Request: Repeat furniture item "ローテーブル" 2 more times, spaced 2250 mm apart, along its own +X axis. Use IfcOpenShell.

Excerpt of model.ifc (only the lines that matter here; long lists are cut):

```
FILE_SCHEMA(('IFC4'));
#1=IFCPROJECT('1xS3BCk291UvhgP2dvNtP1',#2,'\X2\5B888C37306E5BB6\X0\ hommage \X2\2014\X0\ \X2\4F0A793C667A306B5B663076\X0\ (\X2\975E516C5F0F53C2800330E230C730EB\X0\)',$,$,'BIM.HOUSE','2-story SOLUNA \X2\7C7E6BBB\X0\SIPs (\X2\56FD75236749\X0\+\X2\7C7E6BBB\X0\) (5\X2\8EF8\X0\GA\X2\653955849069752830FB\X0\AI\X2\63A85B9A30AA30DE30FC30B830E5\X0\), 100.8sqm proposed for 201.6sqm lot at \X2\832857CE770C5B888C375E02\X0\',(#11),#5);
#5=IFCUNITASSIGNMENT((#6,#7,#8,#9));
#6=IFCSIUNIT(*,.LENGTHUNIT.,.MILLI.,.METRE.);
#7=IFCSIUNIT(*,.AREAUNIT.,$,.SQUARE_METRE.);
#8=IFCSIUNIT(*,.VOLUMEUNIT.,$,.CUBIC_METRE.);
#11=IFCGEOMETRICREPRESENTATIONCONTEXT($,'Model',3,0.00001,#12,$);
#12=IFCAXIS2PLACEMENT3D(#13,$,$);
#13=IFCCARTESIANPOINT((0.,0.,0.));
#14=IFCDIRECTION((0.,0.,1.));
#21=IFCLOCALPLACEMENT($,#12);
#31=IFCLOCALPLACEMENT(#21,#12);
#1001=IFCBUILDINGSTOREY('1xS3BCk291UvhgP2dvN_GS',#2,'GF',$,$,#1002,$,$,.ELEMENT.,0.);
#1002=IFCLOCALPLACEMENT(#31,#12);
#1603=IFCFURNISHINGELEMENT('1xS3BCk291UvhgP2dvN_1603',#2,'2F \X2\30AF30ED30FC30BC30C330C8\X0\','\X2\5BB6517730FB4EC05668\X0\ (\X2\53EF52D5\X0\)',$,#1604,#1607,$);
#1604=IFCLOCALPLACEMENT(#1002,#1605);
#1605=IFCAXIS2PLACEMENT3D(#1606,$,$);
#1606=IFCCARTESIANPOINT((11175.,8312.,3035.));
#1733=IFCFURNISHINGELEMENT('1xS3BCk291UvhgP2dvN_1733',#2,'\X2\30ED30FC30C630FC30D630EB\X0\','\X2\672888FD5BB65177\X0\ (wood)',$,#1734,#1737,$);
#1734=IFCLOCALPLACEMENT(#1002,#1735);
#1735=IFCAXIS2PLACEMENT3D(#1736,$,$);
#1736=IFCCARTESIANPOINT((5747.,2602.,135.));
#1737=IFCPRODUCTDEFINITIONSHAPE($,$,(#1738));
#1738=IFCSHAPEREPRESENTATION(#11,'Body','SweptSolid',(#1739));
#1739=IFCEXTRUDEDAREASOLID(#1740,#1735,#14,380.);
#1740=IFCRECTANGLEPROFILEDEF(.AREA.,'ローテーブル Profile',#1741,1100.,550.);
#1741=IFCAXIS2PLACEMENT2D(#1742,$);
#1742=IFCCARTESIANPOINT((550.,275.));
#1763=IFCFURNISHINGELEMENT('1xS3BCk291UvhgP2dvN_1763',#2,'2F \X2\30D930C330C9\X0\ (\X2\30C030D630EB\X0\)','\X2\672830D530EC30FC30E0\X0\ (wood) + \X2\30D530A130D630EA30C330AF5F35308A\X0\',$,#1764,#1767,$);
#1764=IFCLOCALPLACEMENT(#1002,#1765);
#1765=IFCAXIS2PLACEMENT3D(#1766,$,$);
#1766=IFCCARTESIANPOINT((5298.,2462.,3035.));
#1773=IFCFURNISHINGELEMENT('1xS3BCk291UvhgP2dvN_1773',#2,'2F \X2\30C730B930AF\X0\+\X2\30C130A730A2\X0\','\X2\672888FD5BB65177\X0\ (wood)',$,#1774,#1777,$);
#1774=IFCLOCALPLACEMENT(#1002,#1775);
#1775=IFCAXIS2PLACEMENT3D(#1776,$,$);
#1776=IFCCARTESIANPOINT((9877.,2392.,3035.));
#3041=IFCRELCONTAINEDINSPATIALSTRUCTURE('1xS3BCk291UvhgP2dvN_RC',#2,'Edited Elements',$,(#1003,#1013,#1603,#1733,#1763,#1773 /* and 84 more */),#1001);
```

```python
import ifcopenshell
import ifcopenshell.api.geometry
import ifcopenshell.api.root
import ifcopenshell.util.element
import ifcopenshell.util.placement
import ifcopenshell.util.unit

model = ifcopenshell.open("model.ifc")
unit_scale = ifcopenshell.util.unit.calculate_unit_scale(model)


def reuse_history(source, copy):
    """copy_class also copies each property set's owner history, people and application; keep the originals."""
    for rel in copy.IsDefinedBy:
        if rel.is_a("IfcRelDefinesByProperties") and (history := rel.RelatingPropertyDefinition.OwnerHistory):
            rel.RelatingPropertyDefinition.OwnerHistory = source.OwnerHistory
            ifcopenshell.util.element.remove_deep2(model, history)


source = model.by_id(1733)
base = ifcopenshell.util.placement.get_local_placement(source.ObjectPlacement)
step = base[:3, 0] * 2.25 / unit_scale

for i in range(1, 3):
    copy = ifcopenshell.api.root.copy_class(model, product=source)
    copy.Representation = ifcopenshell.util.element.copy_deep(
        model, source.Representation, exclude=["IfcGeometricRepresentationContext", "IfcRepresentationMap"]
    )
    reuse_history(source, copy)
    matrix = base.copy()
    matrix[:3, 3] += i * step
    print("added at", matrix[:3, 3].round(3) + 0.0)
    ifcopenshell.api.geometry.edit_object_placement(model, product=copy, matrix=matrix, is_si=False)

model.write("model_v2.ifc")
```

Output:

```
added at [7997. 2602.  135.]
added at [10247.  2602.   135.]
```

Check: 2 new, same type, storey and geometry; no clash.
